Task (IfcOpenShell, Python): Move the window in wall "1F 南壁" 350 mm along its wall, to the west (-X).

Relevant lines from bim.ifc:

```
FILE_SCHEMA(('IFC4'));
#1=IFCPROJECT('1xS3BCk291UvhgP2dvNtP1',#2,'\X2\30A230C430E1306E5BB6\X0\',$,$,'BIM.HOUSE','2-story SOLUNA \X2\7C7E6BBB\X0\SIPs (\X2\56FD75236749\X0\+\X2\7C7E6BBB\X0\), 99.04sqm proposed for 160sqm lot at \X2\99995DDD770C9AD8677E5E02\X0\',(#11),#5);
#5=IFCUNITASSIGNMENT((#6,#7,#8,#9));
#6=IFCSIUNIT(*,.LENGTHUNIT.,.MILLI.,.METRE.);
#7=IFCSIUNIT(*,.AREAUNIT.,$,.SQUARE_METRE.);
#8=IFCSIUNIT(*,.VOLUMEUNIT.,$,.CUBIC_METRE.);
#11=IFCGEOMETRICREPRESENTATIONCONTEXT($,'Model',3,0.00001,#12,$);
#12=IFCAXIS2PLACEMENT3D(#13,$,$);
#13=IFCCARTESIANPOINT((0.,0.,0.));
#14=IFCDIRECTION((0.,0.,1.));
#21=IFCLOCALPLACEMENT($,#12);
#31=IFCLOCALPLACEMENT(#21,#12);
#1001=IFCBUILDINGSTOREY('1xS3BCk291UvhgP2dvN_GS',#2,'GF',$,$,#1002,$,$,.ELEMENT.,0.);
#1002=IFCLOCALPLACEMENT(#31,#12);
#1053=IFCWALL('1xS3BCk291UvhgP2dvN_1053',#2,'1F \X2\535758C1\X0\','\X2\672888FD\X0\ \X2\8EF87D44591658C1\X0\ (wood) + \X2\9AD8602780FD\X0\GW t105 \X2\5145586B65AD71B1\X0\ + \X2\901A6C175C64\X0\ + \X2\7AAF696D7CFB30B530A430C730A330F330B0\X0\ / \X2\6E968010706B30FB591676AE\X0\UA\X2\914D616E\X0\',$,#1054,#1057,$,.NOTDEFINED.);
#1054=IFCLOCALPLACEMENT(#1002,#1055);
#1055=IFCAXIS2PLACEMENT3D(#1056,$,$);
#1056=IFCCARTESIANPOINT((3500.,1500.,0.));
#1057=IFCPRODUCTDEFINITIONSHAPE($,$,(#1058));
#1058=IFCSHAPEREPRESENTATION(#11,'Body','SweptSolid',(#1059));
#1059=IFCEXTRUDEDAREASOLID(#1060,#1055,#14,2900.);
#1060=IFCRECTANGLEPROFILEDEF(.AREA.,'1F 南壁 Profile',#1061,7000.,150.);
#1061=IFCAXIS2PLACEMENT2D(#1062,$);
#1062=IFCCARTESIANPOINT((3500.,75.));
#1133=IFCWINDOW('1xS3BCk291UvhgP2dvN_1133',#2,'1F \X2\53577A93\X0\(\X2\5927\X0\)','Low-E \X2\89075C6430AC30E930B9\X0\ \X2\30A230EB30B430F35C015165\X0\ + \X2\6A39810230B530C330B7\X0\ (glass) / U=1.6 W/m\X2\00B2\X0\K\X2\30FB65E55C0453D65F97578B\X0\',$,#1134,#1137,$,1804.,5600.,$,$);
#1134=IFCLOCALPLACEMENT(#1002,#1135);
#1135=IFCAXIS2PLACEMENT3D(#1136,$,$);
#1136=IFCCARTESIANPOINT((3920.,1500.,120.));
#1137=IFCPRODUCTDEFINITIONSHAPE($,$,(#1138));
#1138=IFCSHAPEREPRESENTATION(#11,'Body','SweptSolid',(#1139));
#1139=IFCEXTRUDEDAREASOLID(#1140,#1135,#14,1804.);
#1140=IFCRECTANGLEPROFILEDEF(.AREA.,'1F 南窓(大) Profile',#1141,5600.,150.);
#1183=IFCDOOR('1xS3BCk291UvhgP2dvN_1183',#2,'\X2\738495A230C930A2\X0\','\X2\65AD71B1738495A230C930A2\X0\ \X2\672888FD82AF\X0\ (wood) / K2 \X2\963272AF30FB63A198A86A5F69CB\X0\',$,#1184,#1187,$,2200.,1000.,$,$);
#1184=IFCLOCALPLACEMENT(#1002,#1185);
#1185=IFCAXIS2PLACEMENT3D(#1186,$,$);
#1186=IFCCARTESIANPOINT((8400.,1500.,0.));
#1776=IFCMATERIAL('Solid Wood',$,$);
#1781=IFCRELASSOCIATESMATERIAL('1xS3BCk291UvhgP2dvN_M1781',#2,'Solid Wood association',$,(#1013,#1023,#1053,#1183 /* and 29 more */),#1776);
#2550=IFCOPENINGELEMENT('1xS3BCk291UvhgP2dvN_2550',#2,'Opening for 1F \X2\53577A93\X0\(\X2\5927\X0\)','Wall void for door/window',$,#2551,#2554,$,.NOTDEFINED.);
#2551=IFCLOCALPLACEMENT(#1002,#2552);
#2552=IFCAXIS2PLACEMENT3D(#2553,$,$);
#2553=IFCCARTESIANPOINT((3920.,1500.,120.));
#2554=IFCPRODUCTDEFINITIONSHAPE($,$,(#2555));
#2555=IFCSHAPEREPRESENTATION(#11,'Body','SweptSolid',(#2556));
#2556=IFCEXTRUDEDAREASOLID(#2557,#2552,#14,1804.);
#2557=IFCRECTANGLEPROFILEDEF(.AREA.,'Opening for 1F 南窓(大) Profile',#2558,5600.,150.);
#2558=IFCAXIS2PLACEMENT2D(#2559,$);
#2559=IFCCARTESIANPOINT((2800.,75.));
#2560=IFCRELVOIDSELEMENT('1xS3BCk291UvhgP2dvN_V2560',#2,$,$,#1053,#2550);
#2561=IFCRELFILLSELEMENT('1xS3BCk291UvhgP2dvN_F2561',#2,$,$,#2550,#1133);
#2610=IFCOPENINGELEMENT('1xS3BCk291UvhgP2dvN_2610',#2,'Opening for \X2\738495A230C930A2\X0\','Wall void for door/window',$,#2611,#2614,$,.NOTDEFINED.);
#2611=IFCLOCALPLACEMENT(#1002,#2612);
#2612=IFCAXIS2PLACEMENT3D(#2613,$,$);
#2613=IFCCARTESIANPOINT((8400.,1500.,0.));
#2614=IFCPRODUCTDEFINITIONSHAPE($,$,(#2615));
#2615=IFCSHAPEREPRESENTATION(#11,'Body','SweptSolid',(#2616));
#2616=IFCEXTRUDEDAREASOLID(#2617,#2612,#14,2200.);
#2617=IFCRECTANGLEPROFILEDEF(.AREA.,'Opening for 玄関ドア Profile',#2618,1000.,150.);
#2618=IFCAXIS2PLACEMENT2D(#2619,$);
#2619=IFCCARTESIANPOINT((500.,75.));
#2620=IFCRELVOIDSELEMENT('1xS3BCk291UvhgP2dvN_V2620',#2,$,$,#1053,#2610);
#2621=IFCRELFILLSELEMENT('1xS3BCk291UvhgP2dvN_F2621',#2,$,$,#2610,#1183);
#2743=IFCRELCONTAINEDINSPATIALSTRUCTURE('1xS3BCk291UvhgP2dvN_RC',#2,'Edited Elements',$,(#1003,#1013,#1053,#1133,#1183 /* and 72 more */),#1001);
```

```python
import ifcopenshell
import ifcopenshell.api.geometry
import ifcopenshell.util.placement

model = ifcopenshell.open("bim.ifc")

window = model.by_guid("1xS3BCk291UvhgP2dvN_1133")
opening = window.FillsVoids[0].RelatingOpeningElement
wall = opening.VoidsElements[0].RelatingBuildingElement

wall_matrix = ifcopenshell.util.placement.get_local_placement(wall.ObjectPlacement)
shift = wall_matrix[:3, 0] * -350.0
before = ifcopenshell.util.placement.get_local_placement(window.ObjectPlacement)[:3, 3].copy()

# The window is not placed relative to its opening, so move both.
for product in (opening, window):
    matrix = ifcopenshell.util.placement.get_local_placement(product.ObjectPlacement)
    matrix[:3, 3] += shift
    ifcopenshell.api.geometry.edit_object_placement(model, product=product, matrix=matrix, is_si=False)

after = ifcopenshell.util.placement.get_local_placement(window.ObjectPlacement)[:3, 3]
print("window moved by", (after - before).round(3) + 0.0)

model.write("bim_v2.ifc")
```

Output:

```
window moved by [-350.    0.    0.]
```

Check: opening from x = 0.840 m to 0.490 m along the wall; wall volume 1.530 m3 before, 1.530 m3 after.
